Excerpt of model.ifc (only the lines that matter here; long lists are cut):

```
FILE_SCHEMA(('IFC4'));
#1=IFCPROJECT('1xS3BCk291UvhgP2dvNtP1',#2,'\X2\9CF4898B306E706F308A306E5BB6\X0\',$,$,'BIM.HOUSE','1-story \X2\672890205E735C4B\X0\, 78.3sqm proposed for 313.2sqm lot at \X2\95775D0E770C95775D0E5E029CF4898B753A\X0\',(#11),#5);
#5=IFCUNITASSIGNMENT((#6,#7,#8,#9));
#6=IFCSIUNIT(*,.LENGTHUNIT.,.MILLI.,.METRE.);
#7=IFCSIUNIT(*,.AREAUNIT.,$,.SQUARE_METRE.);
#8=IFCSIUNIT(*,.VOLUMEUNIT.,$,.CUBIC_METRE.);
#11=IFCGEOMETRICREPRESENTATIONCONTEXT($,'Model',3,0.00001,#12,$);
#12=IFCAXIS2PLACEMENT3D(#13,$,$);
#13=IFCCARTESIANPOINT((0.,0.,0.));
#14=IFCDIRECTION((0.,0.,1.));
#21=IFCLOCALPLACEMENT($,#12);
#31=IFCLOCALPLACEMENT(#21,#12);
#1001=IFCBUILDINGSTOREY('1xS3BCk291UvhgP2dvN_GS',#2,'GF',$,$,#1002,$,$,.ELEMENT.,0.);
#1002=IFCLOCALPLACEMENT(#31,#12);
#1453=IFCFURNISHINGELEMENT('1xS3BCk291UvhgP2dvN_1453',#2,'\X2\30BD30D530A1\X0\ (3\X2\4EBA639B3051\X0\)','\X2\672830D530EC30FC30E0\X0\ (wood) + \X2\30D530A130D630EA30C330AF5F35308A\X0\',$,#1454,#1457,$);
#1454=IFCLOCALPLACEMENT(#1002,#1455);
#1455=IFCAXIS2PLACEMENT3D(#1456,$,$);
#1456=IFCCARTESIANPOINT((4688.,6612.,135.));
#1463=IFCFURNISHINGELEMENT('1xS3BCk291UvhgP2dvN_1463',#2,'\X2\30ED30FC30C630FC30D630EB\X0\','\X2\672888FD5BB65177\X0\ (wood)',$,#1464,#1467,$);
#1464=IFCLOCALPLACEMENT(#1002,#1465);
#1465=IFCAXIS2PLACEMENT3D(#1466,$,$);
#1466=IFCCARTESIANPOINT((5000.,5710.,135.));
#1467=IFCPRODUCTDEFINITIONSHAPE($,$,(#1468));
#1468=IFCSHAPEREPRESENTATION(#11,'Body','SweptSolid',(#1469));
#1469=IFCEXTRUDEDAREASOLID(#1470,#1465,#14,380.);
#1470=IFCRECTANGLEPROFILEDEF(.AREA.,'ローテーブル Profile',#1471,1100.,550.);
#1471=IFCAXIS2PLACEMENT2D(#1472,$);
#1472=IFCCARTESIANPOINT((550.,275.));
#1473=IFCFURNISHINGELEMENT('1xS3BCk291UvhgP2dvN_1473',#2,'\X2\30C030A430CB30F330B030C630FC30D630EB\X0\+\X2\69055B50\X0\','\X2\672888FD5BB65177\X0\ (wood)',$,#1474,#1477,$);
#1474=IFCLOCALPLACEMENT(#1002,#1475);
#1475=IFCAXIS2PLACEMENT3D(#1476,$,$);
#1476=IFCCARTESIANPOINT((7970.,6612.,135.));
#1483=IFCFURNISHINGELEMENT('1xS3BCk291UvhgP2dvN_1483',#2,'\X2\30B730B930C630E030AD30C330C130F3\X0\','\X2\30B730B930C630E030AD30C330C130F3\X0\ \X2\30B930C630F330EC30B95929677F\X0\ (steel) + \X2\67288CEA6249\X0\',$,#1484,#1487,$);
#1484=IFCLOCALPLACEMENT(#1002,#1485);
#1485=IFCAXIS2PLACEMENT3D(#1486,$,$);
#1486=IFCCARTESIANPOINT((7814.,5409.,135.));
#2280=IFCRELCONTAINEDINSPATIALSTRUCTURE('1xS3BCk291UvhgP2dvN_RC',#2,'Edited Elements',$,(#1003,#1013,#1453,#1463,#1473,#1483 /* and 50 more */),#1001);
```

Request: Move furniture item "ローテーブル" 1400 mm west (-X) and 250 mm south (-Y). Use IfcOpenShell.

```python
import ifcopenshell
import ifcopenshell.api.geometry
import ifcopenshell.util.placement

model = ifcopenshell.open("model.ifc")

item = model.by_guid("1xS3BCk291UvhgP2dvN_1463")
matrix = ifcopenshell.util.placement.get_local_placement(item.ObjectPlacement)
matrix[0, 3] -= 1400.0
matrix[1, 3] -= 250.0
ifcopenshell.api.geometry.edit_object_placement(model, product=item, matrix=matrix, is_si=False)

print(ifcopenshell.util.placement.get_local_placement(item.ObjectPlacement).round(3) + 0.0)

model.write("model_edited.ifc")
```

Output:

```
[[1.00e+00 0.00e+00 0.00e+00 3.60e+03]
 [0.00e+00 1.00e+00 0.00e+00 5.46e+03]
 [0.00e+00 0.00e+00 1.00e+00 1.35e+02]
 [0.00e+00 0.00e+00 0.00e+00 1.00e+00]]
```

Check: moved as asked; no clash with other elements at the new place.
